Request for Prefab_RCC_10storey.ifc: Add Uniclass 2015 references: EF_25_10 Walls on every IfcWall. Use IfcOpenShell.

First a look at what the model holds.

```python
import ifcopenshell

model = ifcopenshell.open("Prefab_RCC_10storey.ifc")
print(model.schema)
print("classifications:", [c.Name for c in model.by_type("IfcClassification")])
for ifc_class in ("IfcDoor", "IfcRoof", "IfcStair", "IfcWall", "IfcWindow"):
    print(ifc_class, len(model.by_type(ifc_class)))
```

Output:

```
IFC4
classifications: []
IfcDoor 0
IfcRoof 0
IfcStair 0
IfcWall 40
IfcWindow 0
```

```python
import ifcopenshell
import ifcopenshell.api.classification

model = ifcopenshell.open("Prefab_RCC_10storey.ifc")

system = ifcopenshell.api.classification.add_classification(model, classification="Uniclass 2015")

codes = {
    "IfcWall": ("EF_25_10", "Walls"),
}
for ifc_class, (code, name) in codes.items():
    products = model.by_type(ifc_class)
    ifcopenshell.api.classification.add_reference(
        model, products=products, classification=system, identification=code, name=name
    )
    print(code, len(products))

model.write("Prefab_RCC_10storey_v2.ifc")
```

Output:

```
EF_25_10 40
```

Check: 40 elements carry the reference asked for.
